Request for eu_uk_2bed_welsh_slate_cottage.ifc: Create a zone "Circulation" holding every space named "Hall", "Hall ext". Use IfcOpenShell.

First a look at what the model holds.

```python
import ifcopenshell

model = ifcopenshell.open("eu_uk_2bed_welsh_slate_cottage.ifc")
print(model.schema)
seen = {}
for space in model.by_type("IfcSpace"):
    seen[space.LongName] = seen.get(space.LongName, 0) + 1
for name, count in sorted(seen.items(), key=str):
    print(count, "x", name)
print("zones:", [z.Name for z in model.by_type("IfcZone")][:20])
```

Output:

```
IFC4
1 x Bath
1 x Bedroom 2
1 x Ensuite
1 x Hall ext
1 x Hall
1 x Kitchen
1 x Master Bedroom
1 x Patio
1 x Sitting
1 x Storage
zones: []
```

```python
import ifcopenshell
import ifcopenshell.api.group
import ifcopenshell.api.root

model = ifcopenshell.open("eu_uk_2bed_welsh_slate_cottage.ifc")

names = {"Hall", "Hall ext"}
spaces = [s for s in model.by_type("IfcSpace") if s.LongName in names]

zone = ifcopenshell.api.root.create_entity(model, ifc_class="IfcZone", name="Circulation")
ifcopenshell.api.group.assign_group(model, products=spaces, group=zone)
print(len(spaces), "spaces in", zone.Name)

model.write("eu_uk_2bed_welsh_slate_cottage-out.ifc")
```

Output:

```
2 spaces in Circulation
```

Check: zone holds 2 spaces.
